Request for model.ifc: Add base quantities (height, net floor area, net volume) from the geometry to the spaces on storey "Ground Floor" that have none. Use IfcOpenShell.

First a look at what the model holds.

```python
import ifcopenshell
import ifcopenshell.util.element
import ifcopenshell.util.unit

model = ifcopenshell.open("model.ifc")
print(model.schema)
for unit_type in ("LENGTHUNIT", "AREAUNIT", "VOLUMEUNIT"):
    print(unit_type, ifcopenshell.util.unit.calculate_unit_scale(model, unit_type))
storey = next(s for s in model.by_type("IfcBuildingStorey") if s.Name == "Ground Floor")
spaces = [e for e in ifcopenshell.util.element.get_decomposition(storey) if e.is_a("IfcSpace")]
for e in sorted(spaces, key=lambda e: e.id()):
    print(e.id(), e.is_a(), e.Name, list(ifcopenshell.util.element.get_psets(e, qtos_only=True)), sep=" | ")
```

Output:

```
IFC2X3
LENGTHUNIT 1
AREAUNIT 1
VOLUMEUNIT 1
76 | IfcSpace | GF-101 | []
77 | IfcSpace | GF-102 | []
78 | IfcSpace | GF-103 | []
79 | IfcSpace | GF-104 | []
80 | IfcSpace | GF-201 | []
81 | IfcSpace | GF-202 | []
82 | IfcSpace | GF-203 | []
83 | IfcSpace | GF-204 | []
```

```python
import ifcopenshell
import ifcopenshell.api.pset
import ifcopenshell.geom
import ifcopenshell.util.element
import ifcopenshell.util.shape
import ifcopenshell.util.unit

model = ifcopenshell.open("model.ifc")
unit_scale = ifcopenshell.util.unit.calculate_unit_scale(model)
area_scale = ifcopenshell.util.unit.calculate_unit_scale(model, "AREAUNIT")
volume_scale = ifcopenshell.util.unit.calculate_unit_scale(model, "VOLUMEUNIT")
settings = ifcopenshell.geom.settings()

storey = next(s for s in model.by_type("IfcBuildingStorey") if s.Name == "Ground Floor")
spaces = [e for e in ifcopenshell.util.element.get_decomposition(storey) if e.is_a("IfcSpace")]

for e in sorted(spaces, key=lambda e: e.id()):
    if ifcopenshell.util.element.get_psets(e, qtos_only=True, should_inherit=False):
        continue
    # Geometry comes back in metres, in the element's own axes.
    shape = ifcopenshell.geom.create_shape(settings, e)
    values = {
        "Height": ifcopenshell.util.shape.get_z(shape.geometry) / unit_scale,
        "NetFloorArea": ifcopenshell.util.shape.get_footprint_area(shape.geometry) / area_scale,
        "NetVolume": ifcopenshell.util.shape.get_volume(shape.geometry) / volume_scale,
    }
    qto = ifcopenshell.api.pset.add_qto(model, product=e, name="BaseQuantities")
    ifcopenshell.api.pset.edit_qto(model, qto=qto, properties=values)
    print(e.id(), {k: round(v, 3) for k, v in values.items()})

model.write("model_updated.ifc")
```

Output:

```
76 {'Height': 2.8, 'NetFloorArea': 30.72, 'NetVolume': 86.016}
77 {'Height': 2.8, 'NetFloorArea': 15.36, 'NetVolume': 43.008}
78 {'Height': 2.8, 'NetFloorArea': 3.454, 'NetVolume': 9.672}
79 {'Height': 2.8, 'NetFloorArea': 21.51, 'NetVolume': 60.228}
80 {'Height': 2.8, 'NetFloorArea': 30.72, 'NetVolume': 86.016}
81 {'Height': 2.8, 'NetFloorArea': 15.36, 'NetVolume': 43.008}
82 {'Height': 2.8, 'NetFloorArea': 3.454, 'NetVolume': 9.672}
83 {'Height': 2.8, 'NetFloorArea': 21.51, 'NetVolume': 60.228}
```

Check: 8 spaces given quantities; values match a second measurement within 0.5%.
